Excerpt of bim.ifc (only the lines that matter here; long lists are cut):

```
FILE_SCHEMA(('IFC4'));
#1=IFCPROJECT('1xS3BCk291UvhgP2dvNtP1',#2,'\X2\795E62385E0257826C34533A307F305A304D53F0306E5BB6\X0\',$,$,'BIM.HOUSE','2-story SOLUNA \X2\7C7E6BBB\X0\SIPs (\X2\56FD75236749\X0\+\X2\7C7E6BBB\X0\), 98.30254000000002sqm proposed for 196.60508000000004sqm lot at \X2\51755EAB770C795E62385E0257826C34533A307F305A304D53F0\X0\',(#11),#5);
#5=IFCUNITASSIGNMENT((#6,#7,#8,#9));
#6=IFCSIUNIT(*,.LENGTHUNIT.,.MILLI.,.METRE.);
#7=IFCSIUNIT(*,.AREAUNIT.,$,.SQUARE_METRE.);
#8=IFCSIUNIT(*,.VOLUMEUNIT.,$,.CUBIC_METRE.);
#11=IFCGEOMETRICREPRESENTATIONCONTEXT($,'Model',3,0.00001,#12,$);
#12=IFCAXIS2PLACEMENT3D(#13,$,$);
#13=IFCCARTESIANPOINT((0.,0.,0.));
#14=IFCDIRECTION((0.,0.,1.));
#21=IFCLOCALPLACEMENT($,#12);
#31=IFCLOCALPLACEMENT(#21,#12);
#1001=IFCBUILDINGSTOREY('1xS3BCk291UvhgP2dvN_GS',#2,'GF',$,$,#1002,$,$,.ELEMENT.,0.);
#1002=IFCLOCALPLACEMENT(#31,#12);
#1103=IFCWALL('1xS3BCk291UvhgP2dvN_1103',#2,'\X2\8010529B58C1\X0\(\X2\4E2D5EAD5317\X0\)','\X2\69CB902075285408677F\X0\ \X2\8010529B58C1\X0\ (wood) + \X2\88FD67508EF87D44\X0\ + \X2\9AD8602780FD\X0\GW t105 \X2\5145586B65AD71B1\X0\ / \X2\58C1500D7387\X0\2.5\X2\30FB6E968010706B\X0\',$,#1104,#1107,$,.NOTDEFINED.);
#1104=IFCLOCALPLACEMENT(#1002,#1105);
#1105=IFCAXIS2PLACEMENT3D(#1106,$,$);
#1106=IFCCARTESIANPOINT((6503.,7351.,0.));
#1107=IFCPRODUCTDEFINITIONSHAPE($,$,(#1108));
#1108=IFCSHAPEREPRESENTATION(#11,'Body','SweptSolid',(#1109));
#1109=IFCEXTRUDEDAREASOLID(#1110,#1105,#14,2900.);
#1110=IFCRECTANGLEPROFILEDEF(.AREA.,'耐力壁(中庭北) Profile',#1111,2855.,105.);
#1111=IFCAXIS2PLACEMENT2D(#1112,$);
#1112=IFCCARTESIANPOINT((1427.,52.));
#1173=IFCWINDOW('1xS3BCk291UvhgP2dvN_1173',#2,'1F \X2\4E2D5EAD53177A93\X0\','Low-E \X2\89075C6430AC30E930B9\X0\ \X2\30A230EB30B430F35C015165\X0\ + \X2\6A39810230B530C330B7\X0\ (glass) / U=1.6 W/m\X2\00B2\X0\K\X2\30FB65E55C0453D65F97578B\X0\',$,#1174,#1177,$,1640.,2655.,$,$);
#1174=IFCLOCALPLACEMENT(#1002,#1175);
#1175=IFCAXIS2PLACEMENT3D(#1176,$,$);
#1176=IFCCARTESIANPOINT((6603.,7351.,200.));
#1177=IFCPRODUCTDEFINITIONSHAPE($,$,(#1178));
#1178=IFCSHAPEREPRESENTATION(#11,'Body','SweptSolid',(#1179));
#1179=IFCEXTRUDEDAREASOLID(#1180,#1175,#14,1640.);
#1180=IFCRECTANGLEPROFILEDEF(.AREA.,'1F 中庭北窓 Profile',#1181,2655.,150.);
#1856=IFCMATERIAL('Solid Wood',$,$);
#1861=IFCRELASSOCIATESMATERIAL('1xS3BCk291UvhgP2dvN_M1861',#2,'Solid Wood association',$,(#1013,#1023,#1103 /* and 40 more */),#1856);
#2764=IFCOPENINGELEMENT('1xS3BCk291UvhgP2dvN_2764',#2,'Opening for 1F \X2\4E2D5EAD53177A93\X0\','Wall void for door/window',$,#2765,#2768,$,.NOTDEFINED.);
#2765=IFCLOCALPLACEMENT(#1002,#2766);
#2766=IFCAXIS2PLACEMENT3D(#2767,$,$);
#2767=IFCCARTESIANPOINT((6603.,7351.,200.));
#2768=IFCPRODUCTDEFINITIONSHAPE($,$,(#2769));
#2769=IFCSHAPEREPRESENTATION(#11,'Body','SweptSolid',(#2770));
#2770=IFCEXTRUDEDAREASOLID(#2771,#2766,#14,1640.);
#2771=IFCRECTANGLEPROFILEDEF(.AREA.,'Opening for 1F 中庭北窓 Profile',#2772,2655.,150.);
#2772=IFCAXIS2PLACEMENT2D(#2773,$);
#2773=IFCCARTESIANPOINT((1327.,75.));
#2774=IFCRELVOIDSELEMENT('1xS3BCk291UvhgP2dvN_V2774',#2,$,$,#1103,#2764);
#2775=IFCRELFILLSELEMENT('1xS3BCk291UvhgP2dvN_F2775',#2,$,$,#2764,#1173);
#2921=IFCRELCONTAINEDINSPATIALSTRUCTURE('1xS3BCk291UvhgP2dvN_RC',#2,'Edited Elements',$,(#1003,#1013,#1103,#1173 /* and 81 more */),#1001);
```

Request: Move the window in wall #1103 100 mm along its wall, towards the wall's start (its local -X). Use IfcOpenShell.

```python
import ifcopenshell
import ifcopenshell.api.geometry
import ifcopenshell.util.placement
import ifcopenshell.util.unit

model = ifcopenshell.open("bim.ifc")
unit_scale = ifcopenshell.util.unit.calculate_unit_scale(model)

window = model.by_guid("1xS3BCk291UvhgP2dvN_1173")
opening = window.FillsVoids[0].RelatingOpeningElement
wall = opening.VoidsElements[0].RelatingBuildingElement

wall_matrix = ifcopenshell.util.placement.get_local_placement(wall.ObjectPlacement)
shift = wall_matrix[:3, 0] * -0.1 / unit_scale
before = ifcopenshell.util.placement.get_local_placement(window.ObjectPlacement)[:3, 3].copy()

# The window is not placed relative to its opening, so move both.
for product in (opening, window):
    matrix = ifcopenshell.util.placement.get_local_placement(product.ObjectPlacement)
    matrix[:3, 3] += shift
    ifcopenshell.api.geometry.edit_object_placement(model, product=product, matrix=matrix, is_si=False)

after = ifcopenshell.util.placement.get_local_placement(window.ObjectPlacement)[:3, 3]
print("window moved by", (after - before).round(3) + 0.0)

model.write("bim-out.ifc")
```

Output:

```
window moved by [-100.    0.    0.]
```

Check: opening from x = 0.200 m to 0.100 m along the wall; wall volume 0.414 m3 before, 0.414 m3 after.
